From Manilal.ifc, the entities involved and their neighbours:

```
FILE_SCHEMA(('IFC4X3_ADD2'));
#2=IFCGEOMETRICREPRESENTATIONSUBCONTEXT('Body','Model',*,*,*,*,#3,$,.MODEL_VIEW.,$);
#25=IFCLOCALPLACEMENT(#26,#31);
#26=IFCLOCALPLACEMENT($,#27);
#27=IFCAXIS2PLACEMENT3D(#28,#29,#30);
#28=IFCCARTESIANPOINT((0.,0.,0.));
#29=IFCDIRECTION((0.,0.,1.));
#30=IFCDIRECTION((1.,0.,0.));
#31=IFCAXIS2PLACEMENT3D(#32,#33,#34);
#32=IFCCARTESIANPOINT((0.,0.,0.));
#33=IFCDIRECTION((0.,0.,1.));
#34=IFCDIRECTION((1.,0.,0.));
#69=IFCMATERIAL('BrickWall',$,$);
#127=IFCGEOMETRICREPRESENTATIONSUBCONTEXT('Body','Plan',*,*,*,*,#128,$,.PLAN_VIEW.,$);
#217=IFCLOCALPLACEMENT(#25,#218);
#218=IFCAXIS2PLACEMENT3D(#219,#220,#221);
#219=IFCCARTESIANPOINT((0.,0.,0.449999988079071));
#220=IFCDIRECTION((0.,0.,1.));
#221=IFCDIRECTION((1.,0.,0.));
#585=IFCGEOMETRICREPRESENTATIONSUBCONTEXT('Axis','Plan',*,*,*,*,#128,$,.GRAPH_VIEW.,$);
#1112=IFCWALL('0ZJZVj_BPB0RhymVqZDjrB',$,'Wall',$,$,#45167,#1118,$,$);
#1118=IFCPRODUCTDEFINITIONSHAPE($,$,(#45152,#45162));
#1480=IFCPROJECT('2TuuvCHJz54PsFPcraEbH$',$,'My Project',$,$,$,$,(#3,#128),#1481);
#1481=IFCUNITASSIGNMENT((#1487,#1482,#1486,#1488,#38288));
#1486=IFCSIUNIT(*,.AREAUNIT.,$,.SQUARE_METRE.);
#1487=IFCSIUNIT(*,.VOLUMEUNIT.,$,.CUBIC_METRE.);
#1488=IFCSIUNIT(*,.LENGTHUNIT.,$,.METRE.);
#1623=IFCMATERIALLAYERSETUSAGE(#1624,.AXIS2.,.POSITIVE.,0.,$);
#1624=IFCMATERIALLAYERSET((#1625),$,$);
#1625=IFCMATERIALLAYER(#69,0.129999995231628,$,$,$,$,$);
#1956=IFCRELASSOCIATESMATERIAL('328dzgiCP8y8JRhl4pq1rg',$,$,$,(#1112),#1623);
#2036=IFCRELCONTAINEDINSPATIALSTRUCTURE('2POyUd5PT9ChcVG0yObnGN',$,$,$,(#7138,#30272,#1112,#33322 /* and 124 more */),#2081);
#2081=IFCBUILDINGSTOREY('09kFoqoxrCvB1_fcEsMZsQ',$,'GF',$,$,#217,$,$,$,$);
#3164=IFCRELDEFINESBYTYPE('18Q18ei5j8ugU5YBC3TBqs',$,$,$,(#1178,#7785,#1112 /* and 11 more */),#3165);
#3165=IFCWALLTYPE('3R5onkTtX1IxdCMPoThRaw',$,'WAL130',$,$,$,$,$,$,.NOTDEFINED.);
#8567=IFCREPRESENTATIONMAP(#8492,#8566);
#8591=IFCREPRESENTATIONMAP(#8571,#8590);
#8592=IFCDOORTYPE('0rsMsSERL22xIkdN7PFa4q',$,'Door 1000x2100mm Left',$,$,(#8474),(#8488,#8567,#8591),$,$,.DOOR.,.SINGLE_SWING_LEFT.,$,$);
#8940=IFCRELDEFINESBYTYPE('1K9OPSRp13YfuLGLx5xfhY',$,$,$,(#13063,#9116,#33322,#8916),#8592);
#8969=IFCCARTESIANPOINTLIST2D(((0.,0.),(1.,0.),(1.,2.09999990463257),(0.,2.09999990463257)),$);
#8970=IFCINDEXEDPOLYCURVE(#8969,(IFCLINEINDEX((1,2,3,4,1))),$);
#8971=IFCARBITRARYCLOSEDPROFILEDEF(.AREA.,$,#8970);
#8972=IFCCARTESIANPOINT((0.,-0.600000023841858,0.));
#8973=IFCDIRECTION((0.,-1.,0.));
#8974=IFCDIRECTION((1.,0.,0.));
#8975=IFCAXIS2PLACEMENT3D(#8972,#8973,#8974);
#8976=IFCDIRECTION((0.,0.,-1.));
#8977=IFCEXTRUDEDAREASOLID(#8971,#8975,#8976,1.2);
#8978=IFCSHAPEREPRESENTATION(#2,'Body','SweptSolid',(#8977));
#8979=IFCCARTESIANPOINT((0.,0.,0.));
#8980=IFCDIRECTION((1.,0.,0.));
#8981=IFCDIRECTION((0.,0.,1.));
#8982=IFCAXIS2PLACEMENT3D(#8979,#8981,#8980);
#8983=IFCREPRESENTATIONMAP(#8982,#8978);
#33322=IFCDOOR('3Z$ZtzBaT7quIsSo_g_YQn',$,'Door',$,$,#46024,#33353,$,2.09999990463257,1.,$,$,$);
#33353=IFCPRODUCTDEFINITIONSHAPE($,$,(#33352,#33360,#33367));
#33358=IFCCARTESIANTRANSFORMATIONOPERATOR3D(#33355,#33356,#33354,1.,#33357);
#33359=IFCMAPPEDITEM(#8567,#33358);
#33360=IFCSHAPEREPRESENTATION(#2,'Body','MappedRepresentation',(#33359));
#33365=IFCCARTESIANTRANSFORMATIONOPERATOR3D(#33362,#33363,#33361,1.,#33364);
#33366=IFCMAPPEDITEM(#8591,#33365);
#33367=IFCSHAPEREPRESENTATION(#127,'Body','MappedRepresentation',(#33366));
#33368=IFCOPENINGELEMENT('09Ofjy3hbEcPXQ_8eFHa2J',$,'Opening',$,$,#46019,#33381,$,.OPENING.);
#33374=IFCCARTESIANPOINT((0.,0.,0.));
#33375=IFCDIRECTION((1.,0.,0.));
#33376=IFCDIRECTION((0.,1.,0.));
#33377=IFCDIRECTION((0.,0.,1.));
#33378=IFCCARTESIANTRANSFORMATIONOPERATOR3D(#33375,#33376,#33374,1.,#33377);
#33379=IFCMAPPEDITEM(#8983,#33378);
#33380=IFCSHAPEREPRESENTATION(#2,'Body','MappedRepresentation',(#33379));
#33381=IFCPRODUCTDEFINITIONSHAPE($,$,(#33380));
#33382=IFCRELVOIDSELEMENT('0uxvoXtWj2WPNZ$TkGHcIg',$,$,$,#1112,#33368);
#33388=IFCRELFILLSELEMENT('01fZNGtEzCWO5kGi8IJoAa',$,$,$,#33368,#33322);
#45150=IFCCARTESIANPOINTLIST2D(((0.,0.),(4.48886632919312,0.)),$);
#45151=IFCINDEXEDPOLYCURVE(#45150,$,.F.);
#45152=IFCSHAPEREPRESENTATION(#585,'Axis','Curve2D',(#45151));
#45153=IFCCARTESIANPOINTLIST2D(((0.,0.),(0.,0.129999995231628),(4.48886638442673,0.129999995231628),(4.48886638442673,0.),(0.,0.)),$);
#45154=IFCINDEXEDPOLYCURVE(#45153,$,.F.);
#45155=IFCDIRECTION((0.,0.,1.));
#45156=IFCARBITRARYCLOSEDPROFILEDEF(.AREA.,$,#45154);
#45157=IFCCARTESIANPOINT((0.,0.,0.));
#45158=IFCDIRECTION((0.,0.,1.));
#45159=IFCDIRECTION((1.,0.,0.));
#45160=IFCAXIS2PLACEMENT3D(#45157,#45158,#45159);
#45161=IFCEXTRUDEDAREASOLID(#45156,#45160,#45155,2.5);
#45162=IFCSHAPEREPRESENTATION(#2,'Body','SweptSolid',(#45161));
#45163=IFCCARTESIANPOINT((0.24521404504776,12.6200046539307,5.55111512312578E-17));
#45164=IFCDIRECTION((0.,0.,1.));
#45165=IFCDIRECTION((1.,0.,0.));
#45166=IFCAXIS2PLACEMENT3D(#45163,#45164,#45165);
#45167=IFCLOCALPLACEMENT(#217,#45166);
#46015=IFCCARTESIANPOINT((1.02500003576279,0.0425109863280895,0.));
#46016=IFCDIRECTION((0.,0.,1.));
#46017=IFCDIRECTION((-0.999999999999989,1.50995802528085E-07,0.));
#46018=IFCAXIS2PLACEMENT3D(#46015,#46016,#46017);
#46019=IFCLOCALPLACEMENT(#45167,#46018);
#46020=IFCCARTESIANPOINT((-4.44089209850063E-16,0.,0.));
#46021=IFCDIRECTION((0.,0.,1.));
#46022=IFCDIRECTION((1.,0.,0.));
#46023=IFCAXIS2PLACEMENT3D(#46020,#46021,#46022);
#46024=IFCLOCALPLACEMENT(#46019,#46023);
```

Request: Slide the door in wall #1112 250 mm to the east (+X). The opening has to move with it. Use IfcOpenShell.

```python
import ifcopenshell
import ifcopenshell.api.geometry
import ifcopenshell.util.placement

model = ifcopenshell.open("Manilal.ifc")

door = model.by_guid("3Z$ZtzBaT7quIsSo_g_YQn")
opening = door.FillsVoids[0].RelatingOpeningElement
wall = opening.VoidsElements[0].RelatingBuildingElement

wall_matrix = ifcopenshell.util.placement.get_local_placement(wall.ObjectPlacement)
shift = wall_matrix[:3, 0] * 0.25
before = ifcopenshell.util.placement.get_local_placement(door.ObjectPlacement)[:3, 3].copy()

# The door is placed relative to its opening, so it follows when the opening moves.
matrix = ifcopenshell.util.placement.get_local_placement(opening.ObjectPlacement)
matrix[:3, 3] += shift
ifcopenshell.api.geometry.edit_object_placement(
    model, product=opening, matrix=matrix, is_si=False, should_transform_children=True
)

after = ifcopenshell.util.placement.get_local_placement(door.ObjectPlacement)[:3, 3]
print("door moved by", (after - before).round(3) + 0.0)

model.write("Manilal_edited.ifc")
```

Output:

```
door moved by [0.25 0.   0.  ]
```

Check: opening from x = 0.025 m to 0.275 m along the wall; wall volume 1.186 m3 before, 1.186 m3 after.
